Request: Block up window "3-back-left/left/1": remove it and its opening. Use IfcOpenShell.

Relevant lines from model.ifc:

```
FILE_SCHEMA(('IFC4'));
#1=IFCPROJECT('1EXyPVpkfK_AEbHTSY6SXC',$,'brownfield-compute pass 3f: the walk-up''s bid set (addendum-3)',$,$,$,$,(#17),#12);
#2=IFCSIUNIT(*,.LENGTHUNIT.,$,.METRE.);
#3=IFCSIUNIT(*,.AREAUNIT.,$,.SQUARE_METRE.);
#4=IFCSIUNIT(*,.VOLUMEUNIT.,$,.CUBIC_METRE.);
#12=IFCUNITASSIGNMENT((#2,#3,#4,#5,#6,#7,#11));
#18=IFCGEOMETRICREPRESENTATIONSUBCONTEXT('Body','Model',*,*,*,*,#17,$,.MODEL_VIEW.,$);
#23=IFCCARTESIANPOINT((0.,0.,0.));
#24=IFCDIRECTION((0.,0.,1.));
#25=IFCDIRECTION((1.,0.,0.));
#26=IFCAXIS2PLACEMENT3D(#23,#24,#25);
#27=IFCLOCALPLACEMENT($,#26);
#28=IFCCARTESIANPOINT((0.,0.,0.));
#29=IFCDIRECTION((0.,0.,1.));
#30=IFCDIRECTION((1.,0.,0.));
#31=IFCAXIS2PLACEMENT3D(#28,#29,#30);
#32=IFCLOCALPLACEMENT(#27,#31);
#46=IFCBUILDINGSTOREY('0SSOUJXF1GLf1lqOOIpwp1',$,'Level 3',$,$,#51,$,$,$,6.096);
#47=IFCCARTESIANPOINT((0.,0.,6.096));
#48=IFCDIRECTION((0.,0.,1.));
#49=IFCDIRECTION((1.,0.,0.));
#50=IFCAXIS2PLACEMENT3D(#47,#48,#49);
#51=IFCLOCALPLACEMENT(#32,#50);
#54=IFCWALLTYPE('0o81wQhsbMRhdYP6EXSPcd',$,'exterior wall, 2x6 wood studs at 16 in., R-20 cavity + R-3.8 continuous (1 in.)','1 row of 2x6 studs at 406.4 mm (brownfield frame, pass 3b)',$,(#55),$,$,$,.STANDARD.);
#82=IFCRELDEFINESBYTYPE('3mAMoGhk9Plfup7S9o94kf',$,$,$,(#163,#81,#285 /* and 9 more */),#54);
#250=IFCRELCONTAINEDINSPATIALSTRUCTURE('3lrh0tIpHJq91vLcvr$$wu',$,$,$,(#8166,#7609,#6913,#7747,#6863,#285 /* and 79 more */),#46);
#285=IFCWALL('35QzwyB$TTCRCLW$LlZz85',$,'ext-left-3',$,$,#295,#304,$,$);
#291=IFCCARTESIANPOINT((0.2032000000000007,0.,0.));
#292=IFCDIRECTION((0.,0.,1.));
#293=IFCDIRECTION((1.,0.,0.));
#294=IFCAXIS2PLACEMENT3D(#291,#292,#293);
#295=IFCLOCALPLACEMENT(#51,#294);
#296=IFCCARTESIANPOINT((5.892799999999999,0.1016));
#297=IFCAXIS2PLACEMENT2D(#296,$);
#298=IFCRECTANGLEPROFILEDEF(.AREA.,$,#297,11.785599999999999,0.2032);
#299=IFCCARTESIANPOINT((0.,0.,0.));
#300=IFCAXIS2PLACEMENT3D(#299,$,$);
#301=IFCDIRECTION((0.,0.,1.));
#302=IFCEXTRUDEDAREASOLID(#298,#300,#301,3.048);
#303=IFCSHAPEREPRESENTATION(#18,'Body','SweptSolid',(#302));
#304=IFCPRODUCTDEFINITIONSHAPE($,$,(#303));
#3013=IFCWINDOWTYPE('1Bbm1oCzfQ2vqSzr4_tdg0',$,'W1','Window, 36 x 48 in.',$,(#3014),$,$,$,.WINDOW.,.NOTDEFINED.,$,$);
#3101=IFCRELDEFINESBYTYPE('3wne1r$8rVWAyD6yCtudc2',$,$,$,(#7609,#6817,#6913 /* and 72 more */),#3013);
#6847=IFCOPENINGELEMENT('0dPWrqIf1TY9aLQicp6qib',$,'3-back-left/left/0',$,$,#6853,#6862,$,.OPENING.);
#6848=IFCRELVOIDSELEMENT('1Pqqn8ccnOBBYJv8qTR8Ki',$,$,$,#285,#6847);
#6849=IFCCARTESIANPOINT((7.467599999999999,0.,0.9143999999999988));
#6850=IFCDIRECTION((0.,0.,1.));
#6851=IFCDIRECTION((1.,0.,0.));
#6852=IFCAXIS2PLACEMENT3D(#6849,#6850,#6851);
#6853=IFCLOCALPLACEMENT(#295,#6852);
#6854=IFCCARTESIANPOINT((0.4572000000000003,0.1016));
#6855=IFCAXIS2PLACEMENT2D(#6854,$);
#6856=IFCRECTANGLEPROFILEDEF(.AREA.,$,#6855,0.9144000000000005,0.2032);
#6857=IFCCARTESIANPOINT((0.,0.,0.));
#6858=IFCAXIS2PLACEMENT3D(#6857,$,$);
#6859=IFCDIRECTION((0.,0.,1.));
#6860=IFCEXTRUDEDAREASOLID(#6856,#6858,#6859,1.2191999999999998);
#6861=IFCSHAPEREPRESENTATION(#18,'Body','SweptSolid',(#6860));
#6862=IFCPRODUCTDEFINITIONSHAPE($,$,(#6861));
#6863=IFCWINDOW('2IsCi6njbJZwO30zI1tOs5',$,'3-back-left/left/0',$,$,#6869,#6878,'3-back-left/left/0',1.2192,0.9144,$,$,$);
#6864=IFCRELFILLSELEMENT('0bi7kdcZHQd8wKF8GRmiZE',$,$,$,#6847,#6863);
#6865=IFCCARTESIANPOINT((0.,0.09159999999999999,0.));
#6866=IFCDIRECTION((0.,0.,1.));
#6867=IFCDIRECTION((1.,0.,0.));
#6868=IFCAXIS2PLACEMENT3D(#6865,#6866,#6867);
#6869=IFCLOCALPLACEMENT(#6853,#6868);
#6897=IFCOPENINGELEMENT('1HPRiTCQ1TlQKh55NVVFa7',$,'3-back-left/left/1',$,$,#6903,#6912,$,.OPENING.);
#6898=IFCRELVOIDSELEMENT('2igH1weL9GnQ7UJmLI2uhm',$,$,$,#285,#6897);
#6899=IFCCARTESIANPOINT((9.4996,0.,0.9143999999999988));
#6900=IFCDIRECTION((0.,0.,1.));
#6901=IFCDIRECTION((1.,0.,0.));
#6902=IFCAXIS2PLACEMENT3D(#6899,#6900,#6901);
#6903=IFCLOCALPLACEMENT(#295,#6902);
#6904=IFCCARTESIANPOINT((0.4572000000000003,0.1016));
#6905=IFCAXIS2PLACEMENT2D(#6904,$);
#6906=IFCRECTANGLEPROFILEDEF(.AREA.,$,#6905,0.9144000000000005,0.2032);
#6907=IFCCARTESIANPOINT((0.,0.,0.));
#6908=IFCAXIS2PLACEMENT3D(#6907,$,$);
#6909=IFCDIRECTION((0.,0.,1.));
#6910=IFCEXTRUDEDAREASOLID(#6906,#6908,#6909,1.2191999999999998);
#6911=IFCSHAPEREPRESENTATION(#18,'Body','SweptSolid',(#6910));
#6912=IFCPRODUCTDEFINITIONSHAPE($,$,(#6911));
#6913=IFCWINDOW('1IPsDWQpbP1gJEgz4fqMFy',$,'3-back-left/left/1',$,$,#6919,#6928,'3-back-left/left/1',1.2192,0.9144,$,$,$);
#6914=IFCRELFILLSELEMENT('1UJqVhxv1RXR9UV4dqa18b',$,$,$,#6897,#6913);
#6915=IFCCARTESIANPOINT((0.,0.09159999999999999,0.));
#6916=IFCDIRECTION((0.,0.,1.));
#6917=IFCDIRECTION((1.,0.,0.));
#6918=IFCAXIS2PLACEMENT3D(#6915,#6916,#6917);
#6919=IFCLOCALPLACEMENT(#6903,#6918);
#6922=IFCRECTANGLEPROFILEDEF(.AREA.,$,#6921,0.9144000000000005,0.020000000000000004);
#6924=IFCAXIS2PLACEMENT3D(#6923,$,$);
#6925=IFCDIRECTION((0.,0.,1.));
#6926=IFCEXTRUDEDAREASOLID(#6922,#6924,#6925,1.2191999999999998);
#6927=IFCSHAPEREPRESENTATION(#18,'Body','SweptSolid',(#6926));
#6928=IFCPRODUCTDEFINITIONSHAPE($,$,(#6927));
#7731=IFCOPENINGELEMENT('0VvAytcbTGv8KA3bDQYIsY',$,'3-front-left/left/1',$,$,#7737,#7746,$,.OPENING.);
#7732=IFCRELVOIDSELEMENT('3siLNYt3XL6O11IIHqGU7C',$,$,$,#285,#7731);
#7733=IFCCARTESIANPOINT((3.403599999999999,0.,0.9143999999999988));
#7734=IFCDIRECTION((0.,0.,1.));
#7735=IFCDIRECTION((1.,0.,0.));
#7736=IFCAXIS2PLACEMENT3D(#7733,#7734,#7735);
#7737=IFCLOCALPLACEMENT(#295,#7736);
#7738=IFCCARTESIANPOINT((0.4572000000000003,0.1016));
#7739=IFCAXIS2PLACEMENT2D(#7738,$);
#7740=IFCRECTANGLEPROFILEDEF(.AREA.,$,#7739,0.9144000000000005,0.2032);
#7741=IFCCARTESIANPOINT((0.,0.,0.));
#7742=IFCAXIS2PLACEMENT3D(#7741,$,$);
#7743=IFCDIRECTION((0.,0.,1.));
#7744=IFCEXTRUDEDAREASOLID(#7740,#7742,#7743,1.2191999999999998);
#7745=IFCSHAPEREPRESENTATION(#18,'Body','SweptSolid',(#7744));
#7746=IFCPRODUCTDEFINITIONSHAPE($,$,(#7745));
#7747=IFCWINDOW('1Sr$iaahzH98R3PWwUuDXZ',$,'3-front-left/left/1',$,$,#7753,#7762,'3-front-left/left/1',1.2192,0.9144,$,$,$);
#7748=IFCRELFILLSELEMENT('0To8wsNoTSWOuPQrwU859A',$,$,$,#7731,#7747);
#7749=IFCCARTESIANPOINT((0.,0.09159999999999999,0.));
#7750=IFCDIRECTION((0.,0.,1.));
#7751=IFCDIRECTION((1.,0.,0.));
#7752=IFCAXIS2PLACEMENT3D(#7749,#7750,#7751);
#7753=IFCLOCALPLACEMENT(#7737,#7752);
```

```python
import ifcopenshell
import ifcopenshell.api.feature
import ifcopenshell.api.root
import ifcopenshell.geom
import ifcopenshell.util.shape

model = ifcopenshell.open("model.ifc")
settings = ifcopenshell.geom.settings()


def volume(element):
    """Net volume in cubic metres, openings subtracted."""
    shape = ifcopenshell.geom.create_shape(settings, element)
    return ifcopenshell.util.shape.get_volume(shape.geometry)


window = model.by_id(6913)
opening = window.FillsVoids[0].RelatingOpeningElement
wall = opening.VoidsElements[0].RelatingBuildingElement
before = volume(wall)

ifcopenshell.api.root.remove_product(model, product=window)
ifcopenshell.api.feature.remove_feature(model, feature=opening)

after = volume(wall)

print(f"wall volume {before:.3f} -> {after:.3f} m3")

model.write("model_edited.ifc")
```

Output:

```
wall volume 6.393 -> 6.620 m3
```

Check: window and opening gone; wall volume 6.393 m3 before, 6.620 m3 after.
